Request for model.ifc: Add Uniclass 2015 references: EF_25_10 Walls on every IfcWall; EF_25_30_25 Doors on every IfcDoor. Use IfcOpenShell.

First a look at what the model holds.

```python
import ifcopenshell

model = ifcopenshell.open("model.ifc")
print(model.schema)
print("classifications:", [c.Name for c in model.by_type("IfcClassification")])
for ifc_class in ("IfcDoor", "IfcRoof", "IfcStair", "IfcWall", "IfcWindow"):
    print(ifc_class, len(model.by_type(ifc_class)))
```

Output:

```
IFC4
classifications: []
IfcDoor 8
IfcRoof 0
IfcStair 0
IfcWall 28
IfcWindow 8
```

```python
import ifcopenshell
import ifcopenshell.api.classification

model = ifcopenshell.open("model.ifc")

system = ifcopenshell.api.classification.add_classification(model, classification="Uniclass 2015")

codes = {
    "IfcWall": ("EF_25_10", "Walls"),
    "IfcDoor": ("EF_25_30_25", "Doors"),
}
for ifc_class, (code, name) in codes.items():
    products = model.by_type(ifc_class)
    ifcopenshell.api.classification.add_reference(
        model, products=products, classification=system, identification=code, name=name
    )
    print(code, len(products))

model.write("model-out.ifc")
```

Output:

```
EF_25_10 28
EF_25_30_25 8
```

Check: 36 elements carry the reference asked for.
